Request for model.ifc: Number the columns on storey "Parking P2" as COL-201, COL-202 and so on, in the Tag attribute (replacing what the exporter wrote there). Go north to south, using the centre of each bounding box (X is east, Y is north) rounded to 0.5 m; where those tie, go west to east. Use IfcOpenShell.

First a look at what the model holds.

```python
import ifcopenshell
import ifcopenshell.util.element
import ifcopenshell.util.placement

model = ifcopenshell.open("model.ifc")
print(model.schema)
storey = next(s for s in model.by_type("IfcBuildingStorey") if s.Name == "Parking P2")
columns = [e for e in ifcopenshell.util.element.get_decomposition(storey) if e.is_a("IfcColumn")]
for e in sorted(columns, key=lambda e: e.id()):
    origin = ifcopenshell.util.placement.get_local_placement(e.ObjectPlacement)[:3, 3]
    print(e.id(), e.Tag, e.Name, origin.round(2) + 0.0, sep=" | ")
```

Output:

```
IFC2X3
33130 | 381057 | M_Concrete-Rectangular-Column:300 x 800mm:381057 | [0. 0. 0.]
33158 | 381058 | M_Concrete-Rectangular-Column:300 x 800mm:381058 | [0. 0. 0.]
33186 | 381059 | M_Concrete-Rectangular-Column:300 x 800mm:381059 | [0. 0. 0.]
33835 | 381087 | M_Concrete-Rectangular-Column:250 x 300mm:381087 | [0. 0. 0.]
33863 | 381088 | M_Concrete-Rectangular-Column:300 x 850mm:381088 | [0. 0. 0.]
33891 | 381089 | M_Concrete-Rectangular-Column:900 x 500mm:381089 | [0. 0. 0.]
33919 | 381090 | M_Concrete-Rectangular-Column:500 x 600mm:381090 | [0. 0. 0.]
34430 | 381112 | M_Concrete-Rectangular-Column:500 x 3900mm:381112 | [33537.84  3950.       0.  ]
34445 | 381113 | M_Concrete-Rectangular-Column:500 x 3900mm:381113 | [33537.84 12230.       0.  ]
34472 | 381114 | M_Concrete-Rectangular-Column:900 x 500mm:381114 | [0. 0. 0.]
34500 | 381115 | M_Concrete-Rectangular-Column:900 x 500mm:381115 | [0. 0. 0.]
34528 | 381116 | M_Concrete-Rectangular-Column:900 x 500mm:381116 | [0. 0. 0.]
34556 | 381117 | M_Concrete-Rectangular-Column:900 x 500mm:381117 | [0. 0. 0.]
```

```python
import ifcopenshell
import ifcopenshell.geom
import ifcopenshell.util.element
import ifcopenshell.util.shape

model = ifcopenshell.open("model.ifc")
settings = ifcopenshell.geom.settings()
settings.set("use-world-coords", True)


def centre(element):
    shape = ifcopenshell.geom.create_shape(settings, element)
    return ifcopenshell.util.shape.get_bbox_centroid(shape.geometry)


storey = next(s for s in model.by_type("IfcBuildingStorey") if s.Name == "Parking P2")
columns = [e for e in ifcopenshell.util.element.get_decomposition(storey) if e.is_a("IfcColumn")]

# Insertion points can sit at a corner or the storey origin, so sort by the geometry (in metres).
centres = {e: centre(e) for e in columns}
columns.sort(key=lambda e: (-round(centres[e][1] / 0.5), centres[e][0]))

for i, e in enumerate(columns, start=1):
    number = f"COL-2{i:02d}"
    e.Tag = number
    print(e.id(), number)

model.write("model_v2.ifc")
```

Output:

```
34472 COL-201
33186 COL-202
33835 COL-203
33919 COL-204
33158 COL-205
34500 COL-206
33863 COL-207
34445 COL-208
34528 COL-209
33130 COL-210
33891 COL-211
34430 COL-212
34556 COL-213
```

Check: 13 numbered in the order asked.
